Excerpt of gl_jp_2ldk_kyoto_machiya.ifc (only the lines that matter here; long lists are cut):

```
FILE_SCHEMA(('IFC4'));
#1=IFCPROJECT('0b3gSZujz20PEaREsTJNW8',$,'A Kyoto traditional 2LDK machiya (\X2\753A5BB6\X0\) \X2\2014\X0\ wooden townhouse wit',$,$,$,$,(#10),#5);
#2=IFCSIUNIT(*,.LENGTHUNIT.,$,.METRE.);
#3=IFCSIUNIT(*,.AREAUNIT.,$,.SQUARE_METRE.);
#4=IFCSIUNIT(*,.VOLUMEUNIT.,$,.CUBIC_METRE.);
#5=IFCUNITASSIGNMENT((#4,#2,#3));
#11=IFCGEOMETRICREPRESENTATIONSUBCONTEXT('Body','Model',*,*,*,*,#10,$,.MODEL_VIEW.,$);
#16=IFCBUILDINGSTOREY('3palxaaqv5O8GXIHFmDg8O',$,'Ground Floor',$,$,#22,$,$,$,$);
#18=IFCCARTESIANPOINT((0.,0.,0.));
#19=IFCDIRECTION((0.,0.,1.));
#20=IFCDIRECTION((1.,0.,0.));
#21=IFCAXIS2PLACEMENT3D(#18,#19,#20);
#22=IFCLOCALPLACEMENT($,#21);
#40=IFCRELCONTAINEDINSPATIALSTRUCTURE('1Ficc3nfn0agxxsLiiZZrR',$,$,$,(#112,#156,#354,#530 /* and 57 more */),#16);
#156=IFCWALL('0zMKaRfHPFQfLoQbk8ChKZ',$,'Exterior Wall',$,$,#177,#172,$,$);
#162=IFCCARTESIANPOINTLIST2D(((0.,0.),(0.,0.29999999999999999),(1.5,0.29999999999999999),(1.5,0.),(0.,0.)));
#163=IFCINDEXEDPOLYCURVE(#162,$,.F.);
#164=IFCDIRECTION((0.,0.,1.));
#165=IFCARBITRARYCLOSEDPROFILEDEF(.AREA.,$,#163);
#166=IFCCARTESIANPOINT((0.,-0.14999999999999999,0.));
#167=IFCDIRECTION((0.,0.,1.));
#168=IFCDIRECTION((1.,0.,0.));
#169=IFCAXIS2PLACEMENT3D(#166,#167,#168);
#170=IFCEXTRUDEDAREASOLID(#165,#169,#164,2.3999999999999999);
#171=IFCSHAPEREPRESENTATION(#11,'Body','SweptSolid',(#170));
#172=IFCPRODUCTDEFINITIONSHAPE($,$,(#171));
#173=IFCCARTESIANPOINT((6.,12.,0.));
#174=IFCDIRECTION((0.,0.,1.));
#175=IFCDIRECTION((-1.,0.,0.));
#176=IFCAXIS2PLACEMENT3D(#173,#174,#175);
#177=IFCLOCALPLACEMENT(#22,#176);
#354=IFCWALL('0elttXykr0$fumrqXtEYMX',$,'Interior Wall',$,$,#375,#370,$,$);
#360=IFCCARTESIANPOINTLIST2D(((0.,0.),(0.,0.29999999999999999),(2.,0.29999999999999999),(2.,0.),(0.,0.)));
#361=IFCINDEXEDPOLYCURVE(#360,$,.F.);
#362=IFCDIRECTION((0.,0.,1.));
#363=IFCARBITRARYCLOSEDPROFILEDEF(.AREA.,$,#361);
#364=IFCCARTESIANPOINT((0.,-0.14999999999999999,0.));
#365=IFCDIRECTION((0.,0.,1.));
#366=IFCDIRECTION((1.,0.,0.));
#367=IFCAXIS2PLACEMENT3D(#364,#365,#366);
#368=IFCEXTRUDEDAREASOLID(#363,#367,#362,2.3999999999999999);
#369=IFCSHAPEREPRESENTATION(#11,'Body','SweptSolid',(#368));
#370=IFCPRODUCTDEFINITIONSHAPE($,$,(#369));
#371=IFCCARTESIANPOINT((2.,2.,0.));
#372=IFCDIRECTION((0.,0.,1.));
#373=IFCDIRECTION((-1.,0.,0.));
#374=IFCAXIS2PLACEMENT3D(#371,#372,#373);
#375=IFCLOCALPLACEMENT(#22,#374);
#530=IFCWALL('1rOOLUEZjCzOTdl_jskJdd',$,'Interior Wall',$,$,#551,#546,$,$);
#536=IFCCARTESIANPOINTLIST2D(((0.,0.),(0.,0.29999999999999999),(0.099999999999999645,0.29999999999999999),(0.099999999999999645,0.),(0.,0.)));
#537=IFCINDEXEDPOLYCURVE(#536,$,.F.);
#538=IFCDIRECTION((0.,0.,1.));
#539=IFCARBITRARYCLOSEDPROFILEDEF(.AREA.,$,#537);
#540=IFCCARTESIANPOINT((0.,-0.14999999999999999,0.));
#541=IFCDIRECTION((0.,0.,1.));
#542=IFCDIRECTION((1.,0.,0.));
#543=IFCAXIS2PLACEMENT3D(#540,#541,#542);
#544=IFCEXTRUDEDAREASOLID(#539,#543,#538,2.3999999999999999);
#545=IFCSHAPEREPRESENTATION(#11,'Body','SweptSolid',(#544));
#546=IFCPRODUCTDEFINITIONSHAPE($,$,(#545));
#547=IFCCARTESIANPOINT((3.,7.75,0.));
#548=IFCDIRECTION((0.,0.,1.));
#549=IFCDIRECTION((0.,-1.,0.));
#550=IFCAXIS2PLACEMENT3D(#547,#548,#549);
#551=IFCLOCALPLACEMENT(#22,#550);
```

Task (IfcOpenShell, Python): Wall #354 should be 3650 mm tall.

```python
import ifcopenshell
import ifcopenshell.geom
import ifcopenshell.util.representation
import ifcopenshell.util.shape
import ifcopenshell.util.unit

model = ifcopenshell.open("gl_jp_2ldk_kyoto_machiya.ifc")
unit_scale = ifcopenshell.util.unit.calculate_unit_scale(model)
settings = ifcopenshell.geom.settings()


def volume(element):
    """Net volume in cubic metres, openings subtracted."""
    shape = ifcopenshell.geom.create_shape(settings, element)
    return ifcopenshell.util.shape.get_volume(shape.geometry)


wall = model.by_guid("0elttXykr0$fumrqXtEYMX")
before = volume(wall)

body = ifcopenshell.util.representation.get_representation(wall, "Model", "Body")
solid = body.Items[0]
old_height = solid.Depth
solid.Depth = 3.65 / unit_scale
after = volume(wall)

print(f"height {old_height:g} -> {solid.Depth:g}, volume {before:.3f} -> {after:.3f} m3")

model.write("gl_jp_2ldk_kyoto_machiya_v2.ifc")
```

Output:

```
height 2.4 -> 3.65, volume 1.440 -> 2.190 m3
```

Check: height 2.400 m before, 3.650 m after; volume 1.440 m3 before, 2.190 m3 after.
